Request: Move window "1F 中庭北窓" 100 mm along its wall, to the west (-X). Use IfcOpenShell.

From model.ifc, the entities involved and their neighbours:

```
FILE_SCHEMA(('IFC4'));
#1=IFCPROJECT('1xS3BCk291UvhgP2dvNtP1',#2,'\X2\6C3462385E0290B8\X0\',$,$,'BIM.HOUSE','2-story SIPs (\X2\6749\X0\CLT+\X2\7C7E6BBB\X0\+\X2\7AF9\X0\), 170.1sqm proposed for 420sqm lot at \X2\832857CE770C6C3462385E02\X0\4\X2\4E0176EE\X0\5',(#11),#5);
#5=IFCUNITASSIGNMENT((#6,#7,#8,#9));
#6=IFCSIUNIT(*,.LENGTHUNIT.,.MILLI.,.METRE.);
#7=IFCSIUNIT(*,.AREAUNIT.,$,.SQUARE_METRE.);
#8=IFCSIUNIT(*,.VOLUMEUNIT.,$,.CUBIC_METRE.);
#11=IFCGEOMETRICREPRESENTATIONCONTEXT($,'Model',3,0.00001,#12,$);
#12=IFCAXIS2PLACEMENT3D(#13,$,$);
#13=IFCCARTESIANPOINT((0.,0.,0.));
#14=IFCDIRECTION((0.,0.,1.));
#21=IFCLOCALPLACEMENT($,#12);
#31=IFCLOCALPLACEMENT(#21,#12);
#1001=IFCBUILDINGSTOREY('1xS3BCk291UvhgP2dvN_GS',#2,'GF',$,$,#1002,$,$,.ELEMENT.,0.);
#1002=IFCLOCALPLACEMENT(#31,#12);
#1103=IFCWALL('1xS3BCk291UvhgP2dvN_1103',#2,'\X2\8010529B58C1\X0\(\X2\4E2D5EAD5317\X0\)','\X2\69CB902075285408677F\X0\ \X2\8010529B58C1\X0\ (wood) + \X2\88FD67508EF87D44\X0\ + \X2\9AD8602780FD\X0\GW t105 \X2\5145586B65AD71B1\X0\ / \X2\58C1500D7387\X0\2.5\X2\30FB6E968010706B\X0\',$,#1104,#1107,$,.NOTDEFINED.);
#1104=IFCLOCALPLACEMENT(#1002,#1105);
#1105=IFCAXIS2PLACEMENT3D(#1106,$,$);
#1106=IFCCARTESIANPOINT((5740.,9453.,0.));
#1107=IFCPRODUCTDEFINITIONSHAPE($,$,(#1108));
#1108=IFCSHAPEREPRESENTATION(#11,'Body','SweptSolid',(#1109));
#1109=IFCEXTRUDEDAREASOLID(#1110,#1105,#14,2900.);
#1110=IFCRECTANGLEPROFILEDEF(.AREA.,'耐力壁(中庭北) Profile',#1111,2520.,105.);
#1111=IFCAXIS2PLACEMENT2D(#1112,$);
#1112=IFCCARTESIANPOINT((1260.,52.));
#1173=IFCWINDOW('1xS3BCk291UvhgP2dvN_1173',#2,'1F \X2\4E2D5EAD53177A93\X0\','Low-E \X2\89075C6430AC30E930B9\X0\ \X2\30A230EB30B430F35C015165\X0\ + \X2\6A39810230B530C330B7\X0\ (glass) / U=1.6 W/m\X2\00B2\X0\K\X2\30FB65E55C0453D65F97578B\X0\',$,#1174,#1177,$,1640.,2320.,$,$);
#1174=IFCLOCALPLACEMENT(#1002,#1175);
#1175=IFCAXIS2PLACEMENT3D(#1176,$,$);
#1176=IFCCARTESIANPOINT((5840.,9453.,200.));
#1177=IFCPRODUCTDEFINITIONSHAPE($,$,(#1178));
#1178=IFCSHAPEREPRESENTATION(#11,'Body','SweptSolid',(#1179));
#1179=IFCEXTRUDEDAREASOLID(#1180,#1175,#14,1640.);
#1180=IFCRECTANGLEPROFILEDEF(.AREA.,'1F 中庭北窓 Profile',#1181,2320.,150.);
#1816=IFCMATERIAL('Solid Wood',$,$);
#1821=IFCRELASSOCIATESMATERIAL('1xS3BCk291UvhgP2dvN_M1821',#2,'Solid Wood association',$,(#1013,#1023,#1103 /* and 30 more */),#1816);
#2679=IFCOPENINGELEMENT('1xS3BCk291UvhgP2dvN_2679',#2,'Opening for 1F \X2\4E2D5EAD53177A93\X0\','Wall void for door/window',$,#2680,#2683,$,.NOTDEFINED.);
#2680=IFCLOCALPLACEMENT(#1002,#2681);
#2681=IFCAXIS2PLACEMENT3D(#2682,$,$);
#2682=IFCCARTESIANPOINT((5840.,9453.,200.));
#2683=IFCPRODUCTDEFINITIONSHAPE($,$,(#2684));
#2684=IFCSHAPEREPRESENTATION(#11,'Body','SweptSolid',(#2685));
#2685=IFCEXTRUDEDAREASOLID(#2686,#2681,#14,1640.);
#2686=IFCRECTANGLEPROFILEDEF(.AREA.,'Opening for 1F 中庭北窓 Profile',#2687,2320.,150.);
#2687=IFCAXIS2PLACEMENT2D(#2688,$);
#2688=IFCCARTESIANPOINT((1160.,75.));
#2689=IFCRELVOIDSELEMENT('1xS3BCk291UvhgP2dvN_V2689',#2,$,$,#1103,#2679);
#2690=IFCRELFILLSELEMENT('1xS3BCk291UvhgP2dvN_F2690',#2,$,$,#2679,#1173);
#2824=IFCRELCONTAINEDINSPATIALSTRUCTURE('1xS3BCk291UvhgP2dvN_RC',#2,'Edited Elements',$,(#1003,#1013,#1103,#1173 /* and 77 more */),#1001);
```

```python
import ifcopenshell
import ifcopenshell.api.geometry
import ifcopenshell.util.placement
import ifcopenshell.util.unit

model = ifcopenshell.open("model.ifc")
unit_scale = ifcopenshell.util.unit.calculate_unit_scale(model)

window = model.by_guid("1xS3BCk291UvhgP2dvN_1173")
opening = window.FillsVoids[0].RelatingOpeningElement
wall = opening.VoidsElements[0].RelatingBuildingElement

wall_matrix = ifcopenshell.util.placement.get_local_placement(wall.ObjectPlacement)
shift = wall_matrix[:3, 0] * -0.1 / unit_scale
before = ifcopenshell.util.placement.get_local_placement(window.ObjectPlacement)[:3, 3].copy()

# The window is not placed relative to its opening, so move both.
for product in (opening, window):
    matrix = ifcopenshell.util.placement.get_local_placement(product.ObjectPlacement)
    matrix[:3, 3] += shift
    ifcopenshell.api.geometry.edit_object_placement(model, product=product, matrix=matrix, is_si=False)

after = ifcopenshell.util.placement.get_local_placement(window.ObjectPlacement)[:3, 3]
print("window moved by", (after - before).round(3) + 0.0)

model.write("model-out.ifc")
```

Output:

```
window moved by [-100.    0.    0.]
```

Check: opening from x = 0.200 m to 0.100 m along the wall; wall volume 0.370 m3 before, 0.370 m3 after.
